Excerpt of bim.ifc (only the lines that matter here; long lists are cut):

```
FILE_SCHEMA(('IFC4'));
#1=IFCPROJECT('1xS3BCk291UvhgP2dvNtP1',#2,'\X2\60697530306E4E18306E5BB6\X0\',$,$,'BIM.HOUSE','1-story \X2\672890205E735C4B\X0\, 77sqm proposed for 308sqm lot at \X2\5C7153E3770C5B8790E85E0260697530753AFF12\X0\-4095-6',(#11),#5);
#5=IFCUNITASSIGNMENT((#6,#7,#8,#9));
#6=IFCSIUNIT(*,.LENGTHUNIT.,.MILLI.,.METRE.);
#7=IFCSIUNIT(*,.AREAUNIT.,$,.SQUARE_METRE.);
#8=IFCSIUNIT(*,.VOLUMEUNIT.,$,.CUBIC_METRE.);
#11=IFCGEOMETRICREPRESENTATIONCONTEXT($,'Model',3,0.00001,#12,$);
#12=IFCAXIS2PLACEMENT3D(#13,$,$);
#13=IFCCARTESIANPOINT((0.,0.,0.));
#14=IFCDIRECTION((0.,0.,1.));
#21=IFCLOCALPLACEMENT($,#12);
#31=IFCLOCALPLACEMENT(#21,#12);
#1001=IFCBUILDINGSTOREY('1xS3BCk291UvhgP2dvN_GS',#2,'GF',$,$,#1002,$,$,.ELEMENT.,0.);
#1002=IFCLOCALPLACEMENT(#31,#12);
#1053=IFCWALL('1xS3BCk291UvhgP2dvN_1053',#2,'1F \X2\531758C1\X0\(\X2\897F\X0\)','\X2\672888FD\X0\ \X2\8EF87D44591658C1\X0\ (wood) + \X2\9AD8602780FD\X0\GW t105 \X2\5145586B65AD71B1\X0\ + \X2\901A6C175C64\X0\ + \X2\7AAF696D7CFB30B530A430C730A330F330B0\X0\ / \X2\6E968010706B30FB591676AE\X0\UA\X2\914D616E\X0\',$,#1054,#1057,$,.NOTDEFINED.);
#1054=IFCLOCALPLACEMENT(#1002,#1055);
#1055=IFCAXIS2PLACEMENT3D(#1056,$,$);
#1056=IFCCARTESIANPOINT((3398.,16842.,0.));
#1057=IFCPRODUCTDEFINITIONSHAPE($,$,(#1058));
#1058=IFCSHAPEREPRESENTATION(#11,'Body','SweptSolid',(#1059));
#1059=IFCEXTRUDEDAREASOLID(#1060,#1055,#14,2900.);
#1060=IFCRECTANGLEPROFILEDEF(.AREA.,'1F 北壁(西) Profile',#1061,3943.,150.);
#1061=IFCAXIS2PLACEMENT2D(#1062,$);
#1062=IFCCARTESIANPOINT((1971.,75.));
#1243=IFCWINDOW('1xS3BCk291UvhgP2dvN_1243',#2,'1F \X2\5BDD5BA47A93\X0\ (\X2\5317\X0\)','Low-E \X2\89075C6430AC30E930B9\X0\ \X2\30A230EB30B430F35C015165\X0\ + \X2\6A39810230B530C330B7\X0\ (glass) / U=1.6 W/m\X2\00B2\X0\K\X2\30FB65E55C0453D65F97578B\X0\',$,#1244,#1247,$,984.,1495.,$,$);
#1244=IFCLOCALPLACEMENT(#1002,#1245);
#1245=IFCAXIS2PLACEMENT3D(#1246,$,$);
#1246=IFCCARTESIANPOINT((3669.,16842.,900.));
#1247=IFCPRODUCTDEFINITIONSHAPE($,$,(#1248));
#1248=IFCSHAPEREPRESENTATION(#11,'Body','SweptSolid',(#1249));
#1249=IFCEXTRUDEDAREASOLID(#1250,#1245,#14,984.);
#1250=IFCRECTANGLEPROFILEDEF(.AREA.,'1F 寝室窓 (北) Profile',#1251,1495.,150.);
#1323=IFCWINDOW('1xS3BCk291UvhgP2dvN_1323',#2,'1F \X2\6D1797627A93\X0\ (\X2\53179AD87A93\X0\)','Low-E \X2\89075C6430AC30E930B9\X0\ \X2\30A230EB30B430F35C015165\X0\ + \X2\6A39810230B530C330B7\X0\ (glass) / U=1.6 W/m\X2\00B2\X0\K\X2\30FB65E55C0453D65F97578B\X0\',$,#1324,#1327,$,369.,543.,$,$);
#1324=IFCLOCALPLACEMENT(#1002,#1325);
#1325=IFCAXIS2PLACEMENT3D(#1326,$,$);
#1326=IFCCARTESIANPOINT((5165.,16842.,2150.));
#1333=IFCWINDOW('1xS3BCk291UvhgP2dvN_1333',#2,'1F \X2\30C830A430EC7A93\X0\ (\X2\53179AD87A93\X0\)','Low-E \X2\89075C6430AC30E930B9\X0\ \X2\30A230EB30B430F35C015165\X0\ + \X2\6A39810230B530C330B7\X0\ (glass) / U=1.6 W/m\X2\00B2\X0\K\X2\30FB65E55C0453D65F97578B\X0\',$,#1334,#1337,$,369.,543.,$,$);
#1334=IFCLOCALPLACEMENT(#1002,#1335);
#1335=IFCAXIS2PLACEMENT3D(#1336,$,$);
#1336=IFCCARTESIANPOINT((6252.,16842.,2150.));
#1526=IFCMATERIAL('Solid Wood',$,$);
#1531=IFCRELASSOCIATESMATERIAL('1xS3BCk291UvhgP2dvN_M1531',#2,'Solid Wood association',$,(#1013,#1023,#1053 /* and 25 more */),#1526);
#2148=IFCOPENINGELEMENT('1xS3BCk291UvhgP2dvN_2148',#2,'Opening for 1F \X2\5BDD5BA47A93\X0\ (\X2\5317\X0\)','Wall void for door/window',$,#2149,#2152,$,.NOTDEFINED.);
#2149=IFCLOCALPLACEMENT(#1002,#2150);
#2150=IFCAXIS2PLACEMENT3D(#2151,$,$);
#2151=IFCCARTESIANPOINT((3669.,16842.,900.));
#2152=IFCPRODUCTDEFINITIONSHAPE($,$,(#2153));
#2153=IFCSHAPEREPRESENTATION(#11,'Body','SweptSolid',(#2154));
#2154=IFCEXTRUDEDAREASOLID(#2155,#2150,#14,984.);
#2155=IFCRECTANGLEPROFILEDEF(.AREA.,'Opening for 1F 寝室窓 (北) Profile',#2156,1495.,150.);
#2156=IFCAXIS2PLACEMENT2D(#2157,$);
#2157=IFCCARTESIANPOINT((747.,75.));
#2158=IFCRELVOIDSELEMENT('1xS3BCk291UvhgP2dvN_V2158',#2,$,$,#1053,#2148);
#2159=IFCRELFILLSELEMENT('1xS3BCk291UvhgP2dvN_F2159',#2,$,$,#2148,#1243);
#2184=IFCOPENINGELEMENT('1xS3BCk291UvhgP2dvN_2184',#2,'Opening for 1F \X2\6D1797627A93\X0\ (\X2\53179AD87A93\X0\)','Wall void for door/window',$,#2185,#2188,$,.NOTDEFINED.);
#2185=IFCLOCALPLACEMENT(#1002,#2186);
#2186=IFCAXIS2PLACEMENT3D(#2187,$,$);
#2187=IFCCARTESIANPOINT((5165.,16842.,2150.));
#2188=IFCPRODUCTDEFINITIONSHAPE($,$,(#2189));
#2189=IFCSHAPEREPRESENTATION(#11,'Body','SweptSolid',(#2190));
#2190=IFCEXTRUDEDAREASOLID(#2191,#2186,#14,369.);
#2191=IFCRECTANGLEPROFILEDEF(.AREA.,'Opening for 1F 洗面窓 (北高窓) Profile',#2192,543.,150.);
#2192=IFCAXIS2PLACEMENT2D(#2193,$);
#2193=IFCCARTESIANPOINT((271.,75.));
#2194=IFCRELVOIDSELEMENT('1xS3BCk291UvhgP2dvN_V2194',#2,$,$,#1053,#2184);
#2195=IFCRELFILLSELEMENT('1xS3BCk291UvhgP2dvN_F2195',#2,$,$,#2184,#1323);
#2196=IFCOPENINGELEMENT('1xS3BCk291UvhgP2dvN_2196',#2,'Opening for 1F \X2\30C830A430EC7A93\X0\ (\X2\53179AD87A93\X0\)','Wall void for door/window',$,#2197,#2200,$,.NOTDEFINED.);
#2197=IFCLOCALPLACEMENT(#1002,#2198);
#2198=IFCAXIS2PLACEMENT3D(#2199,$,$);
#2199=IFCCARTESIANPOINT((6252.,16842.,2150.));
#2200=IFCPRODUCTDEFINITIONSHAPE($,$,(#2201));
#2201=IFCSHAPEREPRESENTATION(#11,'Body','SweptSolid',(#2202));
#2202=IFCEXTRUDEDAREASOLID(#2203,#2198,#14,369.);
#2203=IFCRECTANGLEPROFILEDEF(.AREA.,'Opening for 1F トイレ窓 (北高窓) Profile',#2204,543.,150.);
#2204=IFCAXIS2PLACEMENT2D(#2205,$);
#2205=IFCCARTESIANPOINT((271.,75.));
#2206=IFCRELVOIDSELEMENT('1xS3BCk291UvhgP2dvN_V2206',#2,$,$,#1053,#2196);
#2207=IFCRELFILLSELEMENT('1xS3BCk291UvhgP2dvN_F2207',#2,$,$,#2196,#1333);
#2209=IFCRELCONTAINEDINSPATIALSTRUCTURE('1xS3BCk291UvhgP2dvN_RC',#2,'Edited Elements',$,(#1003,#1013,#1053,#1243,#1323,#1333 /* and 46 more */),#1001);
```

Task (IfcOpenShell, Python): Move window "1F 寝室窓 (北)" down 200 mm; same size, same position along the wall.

```python
import numpy as np
import ifcopenshell
import ifcopenshell.api.geometry
import ifcopenshell.util.placement
import ifcopenshell.util.unit

model = ifcopenshell.open("bim.ifc")
unit_scale = ifcopenshell.util.unit.calculate_unit_scale(model)

window = model.by_guid("1xS3BCk291UvhgP2dvN_1243")
opening = window.FillsVoids[0].RelatingOpeningElement
dz = -200.0

shift = np.array([0.0, 0.0, dz])
# The window is not placed relative to its opening, so move both.
for product in (opening, window):
    matrix = ifcopenshell.util.placement.get_local_placement(product.ObjectPlacement)
    matrix[:3, 3] += shift
    ifcopenshell.api.geometry.edit_object_placement(model, product=product, matrix=matrix, is_si=False)

print(f"moved by {dz * unit_scale:+.3f} m")

model.write("bim_v2.ifc")
```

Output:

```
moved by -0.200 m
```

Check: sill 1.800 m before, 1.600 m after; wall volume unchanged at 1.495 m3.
